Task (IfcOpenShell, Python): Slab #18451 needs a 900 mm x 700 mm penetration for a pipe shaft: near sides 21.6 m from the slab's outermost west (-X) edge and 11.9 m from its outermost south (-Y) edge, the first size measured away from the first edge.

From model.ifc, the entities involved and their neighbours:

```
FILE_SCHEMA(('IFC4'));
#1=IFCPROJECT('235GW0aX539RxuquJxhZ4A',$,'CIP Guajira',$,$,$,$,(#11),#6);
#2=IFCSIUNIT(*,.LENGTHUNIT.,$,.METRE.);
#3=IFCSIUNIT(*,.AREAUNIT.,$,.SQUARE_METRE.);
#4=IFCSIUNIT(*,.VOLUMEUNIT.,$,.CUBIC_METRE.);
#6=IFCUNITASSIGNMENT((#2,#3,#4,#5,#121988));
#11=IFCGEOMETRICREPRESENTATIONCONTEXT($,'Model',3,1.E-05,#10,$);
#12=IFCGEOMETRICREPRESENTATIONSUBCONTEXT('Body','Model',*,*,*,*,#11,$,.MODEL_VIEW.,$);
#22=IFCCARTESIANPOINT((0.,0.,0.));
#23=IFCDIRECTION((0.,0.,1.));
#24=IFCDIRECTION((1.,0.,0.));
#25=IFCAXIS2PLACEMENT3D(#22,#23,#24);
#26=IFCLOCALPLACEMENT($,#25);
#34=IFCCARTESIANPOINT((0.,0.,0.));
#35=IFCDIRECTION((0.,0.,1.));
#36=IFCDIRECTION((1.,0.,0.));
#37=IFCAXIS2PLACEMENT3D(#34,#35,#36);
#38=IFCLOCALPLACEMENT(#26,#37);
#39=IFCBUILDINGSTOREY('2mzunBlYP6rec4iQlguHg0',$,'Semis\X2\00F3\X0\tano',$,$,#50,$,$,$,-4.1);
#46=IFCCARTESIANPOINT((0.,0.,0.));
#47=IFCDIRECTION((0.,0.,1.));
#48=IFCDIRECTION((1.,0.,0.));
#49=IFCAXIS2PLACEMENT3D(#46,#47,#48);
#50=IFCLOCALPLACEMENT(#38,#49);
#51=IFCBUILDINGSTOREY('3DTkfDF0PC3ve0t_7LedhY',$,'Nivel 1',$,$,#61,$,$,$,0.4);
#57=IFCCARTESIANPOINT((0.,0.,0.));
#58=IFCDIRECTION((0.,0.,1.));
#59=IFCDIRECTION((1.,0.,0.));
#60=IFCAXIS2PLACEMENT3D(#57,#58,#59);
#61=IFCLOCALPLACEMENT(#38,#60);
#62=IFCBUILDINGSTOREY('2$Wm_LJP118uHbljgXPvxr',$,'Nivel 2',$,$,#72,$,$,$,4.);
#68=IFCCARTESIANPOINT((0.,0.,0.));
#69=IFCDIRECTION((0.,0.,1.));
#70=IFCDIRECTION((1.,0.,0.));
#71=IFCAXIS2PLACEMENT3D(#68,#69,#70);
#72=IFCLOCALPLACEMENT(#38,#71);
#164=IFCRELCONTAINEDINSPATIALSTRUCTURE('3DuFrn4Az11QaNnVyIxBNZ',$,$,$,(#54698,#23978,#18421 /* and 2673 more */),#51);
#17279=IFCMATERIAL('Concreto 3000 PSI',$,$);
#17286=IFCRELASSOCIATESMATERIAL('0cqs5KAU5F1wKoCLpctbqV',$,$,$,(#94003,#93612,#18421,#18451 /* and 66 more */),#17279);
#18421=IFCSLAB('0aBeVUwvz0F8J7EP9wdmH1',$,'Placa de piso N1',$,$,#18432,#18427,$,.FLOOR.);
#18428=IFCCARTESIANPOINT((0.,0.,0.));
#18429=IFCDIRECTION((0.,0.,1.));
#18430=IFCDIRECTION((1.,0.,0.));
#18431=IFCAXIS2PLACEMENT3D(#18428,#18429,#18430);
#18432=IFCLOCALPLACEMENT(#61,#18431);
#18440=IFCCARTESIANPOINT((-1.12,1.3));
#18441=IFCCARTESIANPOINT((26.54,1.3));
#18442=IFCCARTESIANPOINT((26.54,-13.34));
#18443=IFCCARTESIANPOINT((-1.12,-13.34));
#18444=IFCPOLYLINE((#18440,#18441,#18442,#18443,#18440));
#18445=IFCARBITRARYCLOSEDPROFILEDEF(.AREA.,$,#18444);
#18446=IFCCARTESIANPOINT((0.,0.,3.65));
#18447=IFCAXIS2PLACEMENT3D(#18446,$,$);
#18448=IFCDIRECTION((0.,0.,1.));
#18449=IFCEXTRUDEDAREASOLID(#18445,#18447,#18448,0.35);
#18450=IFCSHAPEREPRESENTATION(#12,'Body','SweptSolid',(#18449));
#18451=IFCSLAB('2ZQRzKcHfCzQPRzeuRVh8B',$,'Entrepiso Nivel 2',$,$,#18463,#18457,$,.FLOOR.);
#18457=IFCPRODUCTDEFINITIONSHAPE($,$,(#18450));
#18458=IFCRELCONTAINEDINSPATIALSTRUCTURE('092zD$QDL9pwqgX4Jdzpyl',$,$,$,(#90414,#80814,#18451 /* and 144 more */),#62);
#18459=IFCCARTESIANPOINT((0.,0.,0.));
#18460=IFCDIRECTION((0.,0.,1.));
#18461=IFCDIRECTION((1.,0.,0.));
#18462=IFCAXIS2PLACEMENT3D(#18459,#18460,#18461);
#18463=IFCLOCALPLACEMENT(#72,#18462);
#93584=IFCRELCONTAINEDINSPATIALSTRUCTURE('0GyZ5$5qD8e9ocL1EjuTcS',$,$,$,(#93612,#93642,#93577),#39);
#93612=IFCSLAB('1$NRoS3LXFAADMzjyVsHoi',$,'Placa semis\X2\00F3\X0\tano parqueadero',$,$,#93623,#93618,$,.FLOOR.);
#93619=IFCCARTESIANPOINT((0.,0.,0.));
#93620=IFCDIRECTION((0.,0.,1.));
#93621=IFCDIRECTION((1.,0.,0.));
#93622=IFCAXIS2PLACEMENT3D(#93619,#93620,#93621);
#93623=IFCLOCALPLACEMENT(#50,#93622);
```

```python
import numpy as np
import ifcopenshell
import ifcopenshell.api.feature
import ifcopenshell.api.geometry
import ifcopenshell.api.root
import ifcopenshell.geom
import ifcopenshell.util.placement
import ifcopenshell.util.representation
import ifcopenshell.util.shape
import ifcopenshell.util.unit

model = ifcopenshell.open("model.ifc")
unit_scale = ifcopenshell.util.unit.calculate_unit_scale(model)
settings = ifcopenshell.geom.settings()


def volume(element):
    """Net volume in cubic metres, openings subtracted."""
    shape = ifcopenshell.geom.create_shape(settings, element)
    return ifcopenshell.util.shape.get_volume(shape.geometry)


slab = model.by_guid("2ZQRzKcHfCzQPRzeuRVh8B")
before = volume(slab)

# Extent in the slab's own axes, in metres. The edges named are its -X and -Y sides.
slab_shape = ifcopenshell.geom.create_shape(settings, slab)
vertices = ifcopenshell.util.shape.get_vertices(slab_shape.geometry)
x_min, y_min, bottom = vertices.min(axis=0)
top = vertices[:, 2].max()

opening = ifcopenshell.api.root.create_entity(model, ifc_class="IfcOpeningElement", name="Pipe shaft opening", predefined_type="OPENING")
context = ifcopenshell.util.representation.get_context(model, "Model", "Body", "MODEL_VIEW")
width, depth = 0.9, 0.7
outline = [(0.0, 0.0), (width, 0.0), (width, depth), (0.0, depth), (0.0, 0.0)]
# Overshoot both faces by 50 mm so the cut is clean.
shape = ifcopenshell.api.geometry.add_slab_representation(
    model, context=context, depth=top - bottom + 0.1, polyline=outline
)
ifcopenshell.api.geometry.assign_representation(model, product=opening, representation=shape)

matrix = ifcopenshell.util.placement.get_local_placement(slab.ObjectPlacement)
matrix[:, 3] = matrix @ np.append(np.array([x_min + 21.6, y_min + 11.9, bottom - 0.05]) / unit_scale, 1.0)
ifcopenshell.api.geometry.edit_object_placement(model, product=opening, matrix=matrix, is_si=False)
ifcopenshell.api.feature.add_feature(model, feature=opening, element=slab)

after = volume(slab)

print(f"slab volume {before:.3f} -> {after:.3f} m3")

model.write("model_v2.ifc")
```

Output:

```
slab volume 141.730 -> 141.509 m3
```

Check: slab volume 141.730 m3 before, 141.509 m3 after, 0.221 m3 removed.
